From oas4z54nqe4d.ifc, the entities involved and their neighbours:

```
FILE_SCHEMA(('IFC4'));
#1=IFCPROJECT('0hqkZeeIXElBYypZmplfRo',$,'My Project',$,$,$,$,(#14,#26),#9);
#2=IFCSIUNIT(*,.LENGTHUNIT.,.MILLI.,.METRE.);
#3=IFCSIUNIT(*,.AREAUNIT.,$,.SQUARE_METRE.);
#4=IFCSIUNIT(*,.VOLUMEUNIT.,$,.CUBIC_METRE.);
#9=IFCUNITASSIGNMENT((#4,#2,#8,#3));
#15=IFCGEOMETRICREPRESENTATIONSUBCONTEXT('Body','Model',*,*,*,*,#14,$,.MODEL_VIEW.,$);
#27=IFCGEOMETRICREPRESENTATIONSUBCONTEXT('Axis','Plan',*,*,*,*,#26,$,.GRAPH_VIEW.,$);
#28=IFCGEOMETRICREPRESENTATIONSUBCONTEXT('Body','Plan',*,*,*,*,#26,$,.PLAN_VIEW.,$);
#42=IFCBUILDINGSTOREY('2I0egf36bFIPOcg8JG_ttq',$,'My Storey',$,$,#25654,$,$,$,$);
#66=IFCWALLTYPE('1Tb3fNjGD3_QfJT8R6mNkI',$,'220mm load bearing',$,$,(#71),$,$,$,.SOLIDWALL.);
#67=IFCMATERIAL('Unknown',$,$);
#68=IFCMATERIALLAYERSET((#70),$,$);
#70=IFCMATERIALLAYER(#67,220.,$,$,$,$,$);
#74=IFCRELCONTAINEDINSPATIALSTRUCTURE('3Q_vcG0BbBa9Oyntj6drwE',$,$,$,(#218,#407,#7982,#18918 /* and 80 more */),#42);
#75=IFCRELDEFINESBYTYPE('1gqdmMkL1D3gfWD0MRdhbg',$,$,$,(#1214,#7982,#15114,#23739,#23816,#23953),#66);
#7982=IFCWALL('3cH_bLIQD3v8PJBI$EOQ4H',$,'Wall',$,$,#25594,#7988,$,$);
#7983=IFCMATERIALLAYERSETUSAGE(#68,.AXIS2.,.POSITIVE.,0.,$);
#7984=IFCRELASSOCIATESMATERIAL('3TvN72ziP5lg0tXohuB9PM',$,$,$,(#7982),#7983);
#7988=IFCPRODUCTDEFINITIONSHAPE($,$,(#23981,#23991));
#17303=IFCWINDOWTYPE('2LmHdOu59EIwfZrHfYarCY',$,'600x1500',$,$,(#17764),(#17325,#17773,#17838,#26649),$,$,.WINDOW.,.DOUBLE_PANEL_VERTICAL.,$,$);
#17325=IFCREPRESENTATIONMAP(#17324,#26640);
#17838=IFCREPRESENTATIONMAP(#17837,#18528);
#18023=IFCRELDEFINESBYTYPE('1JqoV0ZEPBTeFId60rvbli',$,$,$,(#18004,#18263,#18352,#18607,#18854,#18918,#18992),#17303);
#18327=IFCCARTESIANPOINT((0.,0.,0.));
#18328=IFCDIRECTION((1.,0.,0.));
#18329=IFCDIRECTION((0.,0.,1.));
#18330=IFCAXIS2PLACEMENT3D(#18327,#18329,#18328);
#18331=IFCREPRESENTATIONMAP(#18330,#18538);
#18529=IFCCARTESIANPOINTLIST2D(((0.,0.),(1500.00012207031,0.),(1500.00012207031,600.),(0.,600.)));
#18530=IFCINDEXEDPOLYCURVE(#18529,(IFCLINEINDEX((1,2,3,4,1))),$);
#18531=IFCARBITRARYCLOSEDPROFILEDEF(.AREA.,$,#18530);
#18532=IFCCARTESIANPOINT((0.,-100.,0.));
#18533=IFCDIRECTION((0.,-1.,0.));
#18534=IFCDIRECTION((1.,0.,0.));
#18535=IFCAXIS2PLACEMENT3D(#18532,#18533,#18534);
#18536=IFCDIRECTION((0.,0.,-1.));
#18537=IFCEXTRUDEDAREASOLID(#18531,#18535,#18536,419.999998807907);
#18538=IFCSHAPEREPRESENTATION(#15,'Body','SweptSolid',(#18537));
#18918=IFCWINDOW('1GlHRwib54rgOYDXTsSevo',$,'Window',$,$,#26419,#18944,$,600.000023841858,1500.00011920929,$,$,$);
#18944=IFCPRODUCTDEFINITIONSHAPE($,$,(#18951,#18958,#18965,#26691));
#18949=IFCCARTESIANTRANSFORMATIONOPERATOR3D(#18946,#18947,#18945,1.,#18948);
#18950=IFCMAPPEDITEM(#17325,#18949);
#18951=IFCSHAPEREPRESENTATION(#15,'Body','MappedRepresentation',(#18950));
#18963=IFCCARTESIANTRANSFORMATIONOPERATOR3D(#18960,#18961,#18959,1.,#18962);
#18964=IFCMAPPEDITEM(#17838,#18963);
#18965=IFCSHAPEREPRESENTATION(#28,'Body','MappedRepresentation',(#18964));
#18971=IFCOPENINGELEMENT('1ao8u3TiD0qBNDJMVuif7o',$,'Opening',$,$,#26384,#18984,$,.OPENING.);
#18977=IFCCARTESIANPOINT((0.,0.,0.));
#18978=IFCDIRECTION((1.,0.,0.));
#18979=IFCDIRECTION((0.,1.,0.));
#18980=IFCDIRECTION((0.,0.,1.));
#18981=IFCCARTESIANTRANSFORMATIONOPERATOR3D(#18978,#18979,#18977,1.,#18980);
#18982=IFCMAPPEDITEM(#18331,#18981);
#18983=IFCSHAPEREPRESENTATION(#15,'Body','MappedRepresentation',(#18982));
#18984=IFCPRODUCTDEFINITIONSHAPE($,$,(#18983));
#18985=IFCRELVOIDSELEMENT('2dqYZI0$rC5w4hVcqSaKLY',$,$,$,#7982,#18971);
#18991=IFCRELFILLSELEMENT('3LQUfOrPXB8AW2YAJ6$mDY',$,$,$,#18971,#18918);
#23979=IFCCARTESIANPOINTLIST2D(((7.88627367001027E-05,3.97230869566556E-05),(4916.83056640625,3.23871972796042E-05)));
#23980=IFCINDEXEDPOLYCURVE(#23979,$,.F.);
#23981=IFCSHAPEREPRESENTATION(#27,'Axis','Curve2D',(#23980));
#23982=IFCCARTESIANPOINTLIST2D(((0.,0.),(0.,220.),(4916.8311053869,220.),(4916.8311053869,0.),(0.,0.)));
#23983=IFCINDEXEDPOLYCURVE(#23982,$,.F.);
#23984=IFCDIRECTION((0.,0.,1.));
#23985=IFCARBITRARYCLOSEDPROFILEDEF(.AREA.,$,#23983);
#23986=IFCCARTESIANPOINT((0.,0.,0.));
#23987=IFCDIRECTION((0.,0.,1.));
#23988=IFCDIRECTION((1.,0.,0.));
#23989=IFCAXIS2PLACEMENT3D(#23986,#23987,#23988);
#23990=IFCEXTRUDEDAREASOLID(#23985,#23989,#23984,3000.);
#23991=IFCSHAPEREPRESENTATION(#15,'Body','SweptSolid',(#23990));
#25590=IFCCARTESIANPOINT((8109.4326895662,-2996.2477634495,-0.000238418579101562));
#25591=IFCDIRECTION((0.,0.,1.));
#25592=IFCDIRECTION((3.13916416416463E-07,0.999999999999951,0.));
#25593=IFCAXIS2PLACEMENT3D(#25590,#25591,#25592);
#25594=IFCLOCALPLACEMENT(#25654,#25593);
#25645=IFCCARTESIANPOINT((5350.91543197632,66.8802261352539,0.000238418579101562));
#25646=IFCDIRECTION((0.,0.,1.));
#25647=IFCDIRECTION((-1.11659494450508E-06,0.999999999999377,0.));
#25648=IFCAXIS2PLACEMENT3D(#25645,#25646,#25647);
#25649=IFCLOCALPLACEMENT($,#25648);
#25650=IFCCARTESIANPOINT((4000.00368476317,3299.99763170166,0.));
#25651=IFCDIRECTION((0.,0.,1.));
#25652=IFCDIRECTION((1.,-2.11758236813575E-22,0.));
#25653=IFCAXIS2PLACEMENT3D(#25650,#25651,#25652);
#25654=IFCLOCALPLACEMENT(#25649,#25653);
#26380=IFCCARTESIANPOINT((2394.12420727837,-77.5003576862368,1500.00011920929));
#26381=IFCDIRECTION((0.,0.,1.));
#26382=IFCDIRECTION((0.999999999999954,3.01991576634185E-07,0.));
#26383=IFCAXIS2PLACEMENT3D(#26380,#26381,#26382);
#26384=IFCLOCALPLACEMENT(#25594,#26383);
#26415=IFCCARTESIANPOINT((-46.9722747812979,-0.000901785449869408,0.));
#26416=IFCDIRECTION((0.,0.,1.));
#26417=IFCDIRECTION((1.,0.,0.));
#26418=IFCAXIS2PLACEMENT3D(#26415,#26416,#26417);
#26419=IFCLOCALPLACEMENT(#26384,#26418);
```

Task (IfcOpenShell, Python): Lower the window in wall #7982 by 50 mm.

```python
import numpy as np
import ifcopenshell
import ifcopenshell.api.geometry
import ifcopenshell.util.placement
import ifcopenshell.util.unit

model = ifcopenshell.open("oas4z54nqe4d.ifc")
unit_scale = ifcopenshell.util.unit.calculate_unit_scale(model)

window = model.by_guid("1GlHRwib54rgOYDXTsSevo")
opening = window.FillsVoids[0].RelatingOpeningElement
dz = -0.05 / unit_scale

shift = np.array([0.0, 0.0, dz])
# The window is placed relative to its opening, so it follows when the opening moves.
matrix = ifcopenshell.util.placement.get_local_placement(opening.ObjectPlacement)
matrix[:3, 3] += shift
ifcopenshell.api.geometry.edit_object_placement(
    model, product=opening, matrix=matrix, is_si=False, should_transform_children=True
)

print(f"moved by {dz * unit_scale:+.3f} m")

model.write("oas4z54nqe4d_rev.ifc")
```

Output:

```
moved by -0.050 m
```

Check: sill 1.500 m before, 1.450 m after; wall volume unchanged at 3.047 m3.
